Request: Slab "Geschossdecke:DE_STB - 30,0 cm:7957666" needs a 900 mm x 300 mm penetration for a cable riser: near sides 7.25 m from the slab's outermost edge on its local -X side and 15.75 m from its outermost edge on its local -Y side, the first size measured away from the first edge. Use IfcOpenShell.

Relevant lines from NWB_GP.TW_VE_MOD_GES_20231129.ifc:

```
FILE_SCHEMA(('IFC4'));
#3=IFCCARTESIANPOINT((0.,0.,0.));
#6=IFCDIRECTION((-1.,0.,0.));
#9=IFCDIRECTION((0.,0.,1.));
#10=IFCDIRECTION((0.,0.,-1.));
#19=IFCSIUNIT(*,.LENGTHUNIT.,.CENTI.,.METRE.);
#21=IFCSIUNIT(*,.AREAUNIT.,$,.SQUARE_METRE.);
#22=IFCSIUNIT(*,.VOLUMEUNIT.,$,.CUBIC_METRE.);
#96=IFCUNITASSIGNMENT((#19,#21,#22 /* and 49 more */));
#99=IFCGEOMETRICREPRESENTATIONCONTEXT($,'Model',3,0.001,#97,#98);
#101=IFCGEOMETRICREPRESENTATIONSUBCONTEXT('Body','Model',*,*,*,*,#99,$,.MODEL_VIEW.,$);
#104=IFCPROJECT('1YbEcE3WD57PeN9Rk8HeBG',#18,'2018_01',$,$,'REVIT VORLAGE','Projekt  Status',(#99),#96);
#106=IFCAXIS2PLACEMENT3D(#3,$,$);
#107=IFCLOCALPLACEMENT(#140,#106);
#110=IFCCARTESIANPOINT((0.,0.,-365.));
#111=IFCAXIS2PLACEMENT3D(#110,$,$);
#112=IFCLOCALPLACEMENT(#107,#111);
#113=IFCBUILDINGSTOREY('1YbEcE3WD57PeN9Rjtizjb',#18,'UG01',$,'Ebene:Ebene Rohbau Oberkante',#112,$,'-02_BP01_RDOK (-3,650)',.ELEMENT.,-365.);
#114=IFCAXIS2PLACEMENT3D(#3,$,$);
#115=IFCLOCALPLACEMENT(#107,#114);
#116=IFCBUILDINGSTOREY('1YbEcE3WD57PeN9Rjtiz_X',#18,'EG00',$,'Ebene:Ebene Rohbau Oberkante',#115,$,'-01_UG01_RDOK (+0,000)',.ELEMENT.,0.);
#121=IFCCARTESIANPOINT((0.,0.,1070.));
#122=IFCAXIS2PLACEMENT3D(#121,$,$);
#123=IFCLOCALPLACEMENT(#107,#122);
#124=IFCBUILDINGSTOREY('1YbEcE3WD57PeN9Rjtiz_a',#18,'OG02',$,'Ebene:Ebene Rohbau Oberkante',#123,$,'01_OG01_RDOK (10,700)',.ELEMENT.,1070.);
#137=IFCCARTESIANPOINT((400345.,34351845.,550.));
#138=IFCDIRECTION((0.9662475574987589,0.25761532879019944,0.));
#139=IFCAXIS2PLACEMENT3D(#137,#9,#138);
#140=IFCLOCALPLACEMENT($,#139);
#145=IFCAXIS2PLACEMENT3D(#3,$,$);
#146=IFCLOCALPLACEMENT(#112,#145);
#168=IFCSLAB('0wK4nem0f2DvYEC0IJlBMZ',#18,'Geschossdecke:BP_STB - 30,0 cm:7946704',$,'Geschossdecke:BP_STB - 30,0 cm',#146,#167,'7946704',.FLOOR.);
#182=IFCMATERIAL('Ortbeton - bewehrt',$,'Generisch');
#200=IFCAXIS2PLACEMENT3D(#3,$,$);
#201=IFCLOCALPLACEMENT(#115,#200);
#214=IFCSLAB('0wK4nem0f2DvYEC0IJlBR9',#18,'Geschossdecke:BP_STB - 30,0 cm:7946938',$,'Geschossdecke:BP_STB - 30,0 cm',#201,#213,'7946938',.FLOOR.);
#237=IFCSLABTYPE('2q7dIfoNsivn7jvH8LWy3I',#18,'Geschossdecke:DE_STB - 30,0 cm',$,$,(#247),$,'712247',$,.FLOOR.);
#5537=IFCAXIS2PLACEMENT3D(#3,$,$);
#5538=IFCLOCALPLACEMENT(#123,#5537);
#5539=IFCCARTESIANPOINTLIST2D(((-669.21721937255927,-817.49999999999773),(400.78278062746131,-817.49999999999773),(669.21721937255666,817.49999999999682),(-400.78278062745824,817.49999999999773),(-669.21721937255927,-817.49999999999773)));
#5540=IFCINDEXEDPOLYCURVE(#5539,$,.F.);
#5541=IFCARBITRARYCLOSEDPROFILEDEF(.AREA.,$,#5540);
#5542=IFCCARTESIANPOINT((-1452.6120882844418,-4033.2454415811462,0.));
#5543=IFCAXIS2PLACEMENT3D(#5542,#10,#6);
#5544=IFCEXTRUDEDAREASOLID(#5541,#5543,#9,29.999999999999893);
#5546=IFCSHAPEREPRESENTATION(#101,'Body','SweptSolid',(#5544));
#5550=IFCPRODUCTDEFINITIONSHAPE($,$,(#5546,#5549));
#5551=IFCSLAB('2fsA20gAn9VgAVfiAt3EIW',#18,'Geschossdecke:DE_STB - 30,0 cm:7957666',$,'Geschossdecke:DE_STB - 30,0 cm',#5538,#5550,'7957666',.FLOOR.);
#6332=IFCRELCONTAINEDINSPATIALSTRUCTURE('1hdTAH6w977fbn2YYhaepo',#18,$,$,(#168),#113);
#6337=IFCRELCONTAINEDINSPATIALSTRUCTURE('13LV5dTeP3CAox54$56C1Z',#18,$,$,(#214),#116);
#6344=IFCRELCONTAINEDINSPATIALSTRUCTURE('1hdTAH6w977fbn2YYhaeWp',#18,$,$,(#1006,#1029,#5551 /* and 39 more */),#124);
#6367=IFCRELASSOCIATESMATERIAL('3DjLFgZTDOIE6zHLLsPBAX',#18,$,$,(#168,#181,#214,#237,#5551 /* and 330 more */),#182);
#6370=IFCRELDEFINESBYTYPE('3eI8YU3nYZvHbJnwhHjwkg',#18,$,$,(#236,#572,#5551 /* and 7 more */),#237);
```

```python
import numpy as np
import ifcopenshell
import ifcopenshell.api.feature
import ifcopenshell.api.geometry
import ifcopenshell.api.root
import ifcopenshell.geom
import ifcopenshell.util.placement
import ifcopenshell.util.representation
import ifcopenshell.util.shape
import ifcopenshell.util.unit

model = ifcopenshell.open("NWB_GP.TW_VE_MOD_GES_20231129.ifc")
unit_scale = ifcopenshell.util.unit.calculate_unit_scale(model)
settings = ifcopenshell.geom.settings()


def volume(element):
    """Net volume in cubic metres, openings subtracted."""
    shape = ifcopenshell.geom.create_shape(settings, element)
    return ifcopenshell.util.shape.get_volume(shape.geometry)


slab = model.by_guid("2fsA20gAn9VgAVfiAt3EIW")
before = volume(slab)

# Extent in the slab's own axes, in metres. The edges named are its -X and -Y sides.
slab_shape = ifcopenshell.geom.create_shape(settings, slab)
vertices = ifcopenshell.util.shape.get_vertices(slab_shape.geometry)
x_min, y_min, bottom = vertices.min(axis=0)
top = vertices[:, 2].max()

opening = ifcopenshell.api.root.create_entity(model, ifc_class="IfcOpeningElement", name="Cable riser opening", predefined_type="OPENING")
context = ifcopenshell.util.representation.get_context(model, "Model", "Body", "MODEL_VIEW")
width, depth = 0.9, 0.3
outline = [(0.0, 0.0), (width, 0.0), (width, depth), (0.0, depth), (0.0, 0.0)]
# Overshoot both faces by 50 mm so the cut is clean.
shape = ifcopenshell.api.geometry.add_slab_representation(
    model, context=context, depth=top - bottom + 0.1, polyline=outline
)
ifcopenshell.api.geometry.assign_representation(model, product=opening, representation=shape)

matrix = ifcopenshell.util.placement.get_local_placement(slab.ObjectPlacement)
matrix[:, 3] = matrix @ np.append(np.array([x_min + 7.25, y_min + 15.75, bottom - 0.05]) / unit_scale, 1.0)
ifcopenshell.api.geometry.edit_object_placement(model, product=opening, matrix=matrix, is_si=False)
ifcopenshell.api.feature.add_feature(model, feature=opening, element=slab)

after = volume(slab)

print(f"slab volume {before:.3f} -> {after:.3f} m3")

model.write("NWB_GP.TW_VE_MOD_GES_20231129-out.ifc")
```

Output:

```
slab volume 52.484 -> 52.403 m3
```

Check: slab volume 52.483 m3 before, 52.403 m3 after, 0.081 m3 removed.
